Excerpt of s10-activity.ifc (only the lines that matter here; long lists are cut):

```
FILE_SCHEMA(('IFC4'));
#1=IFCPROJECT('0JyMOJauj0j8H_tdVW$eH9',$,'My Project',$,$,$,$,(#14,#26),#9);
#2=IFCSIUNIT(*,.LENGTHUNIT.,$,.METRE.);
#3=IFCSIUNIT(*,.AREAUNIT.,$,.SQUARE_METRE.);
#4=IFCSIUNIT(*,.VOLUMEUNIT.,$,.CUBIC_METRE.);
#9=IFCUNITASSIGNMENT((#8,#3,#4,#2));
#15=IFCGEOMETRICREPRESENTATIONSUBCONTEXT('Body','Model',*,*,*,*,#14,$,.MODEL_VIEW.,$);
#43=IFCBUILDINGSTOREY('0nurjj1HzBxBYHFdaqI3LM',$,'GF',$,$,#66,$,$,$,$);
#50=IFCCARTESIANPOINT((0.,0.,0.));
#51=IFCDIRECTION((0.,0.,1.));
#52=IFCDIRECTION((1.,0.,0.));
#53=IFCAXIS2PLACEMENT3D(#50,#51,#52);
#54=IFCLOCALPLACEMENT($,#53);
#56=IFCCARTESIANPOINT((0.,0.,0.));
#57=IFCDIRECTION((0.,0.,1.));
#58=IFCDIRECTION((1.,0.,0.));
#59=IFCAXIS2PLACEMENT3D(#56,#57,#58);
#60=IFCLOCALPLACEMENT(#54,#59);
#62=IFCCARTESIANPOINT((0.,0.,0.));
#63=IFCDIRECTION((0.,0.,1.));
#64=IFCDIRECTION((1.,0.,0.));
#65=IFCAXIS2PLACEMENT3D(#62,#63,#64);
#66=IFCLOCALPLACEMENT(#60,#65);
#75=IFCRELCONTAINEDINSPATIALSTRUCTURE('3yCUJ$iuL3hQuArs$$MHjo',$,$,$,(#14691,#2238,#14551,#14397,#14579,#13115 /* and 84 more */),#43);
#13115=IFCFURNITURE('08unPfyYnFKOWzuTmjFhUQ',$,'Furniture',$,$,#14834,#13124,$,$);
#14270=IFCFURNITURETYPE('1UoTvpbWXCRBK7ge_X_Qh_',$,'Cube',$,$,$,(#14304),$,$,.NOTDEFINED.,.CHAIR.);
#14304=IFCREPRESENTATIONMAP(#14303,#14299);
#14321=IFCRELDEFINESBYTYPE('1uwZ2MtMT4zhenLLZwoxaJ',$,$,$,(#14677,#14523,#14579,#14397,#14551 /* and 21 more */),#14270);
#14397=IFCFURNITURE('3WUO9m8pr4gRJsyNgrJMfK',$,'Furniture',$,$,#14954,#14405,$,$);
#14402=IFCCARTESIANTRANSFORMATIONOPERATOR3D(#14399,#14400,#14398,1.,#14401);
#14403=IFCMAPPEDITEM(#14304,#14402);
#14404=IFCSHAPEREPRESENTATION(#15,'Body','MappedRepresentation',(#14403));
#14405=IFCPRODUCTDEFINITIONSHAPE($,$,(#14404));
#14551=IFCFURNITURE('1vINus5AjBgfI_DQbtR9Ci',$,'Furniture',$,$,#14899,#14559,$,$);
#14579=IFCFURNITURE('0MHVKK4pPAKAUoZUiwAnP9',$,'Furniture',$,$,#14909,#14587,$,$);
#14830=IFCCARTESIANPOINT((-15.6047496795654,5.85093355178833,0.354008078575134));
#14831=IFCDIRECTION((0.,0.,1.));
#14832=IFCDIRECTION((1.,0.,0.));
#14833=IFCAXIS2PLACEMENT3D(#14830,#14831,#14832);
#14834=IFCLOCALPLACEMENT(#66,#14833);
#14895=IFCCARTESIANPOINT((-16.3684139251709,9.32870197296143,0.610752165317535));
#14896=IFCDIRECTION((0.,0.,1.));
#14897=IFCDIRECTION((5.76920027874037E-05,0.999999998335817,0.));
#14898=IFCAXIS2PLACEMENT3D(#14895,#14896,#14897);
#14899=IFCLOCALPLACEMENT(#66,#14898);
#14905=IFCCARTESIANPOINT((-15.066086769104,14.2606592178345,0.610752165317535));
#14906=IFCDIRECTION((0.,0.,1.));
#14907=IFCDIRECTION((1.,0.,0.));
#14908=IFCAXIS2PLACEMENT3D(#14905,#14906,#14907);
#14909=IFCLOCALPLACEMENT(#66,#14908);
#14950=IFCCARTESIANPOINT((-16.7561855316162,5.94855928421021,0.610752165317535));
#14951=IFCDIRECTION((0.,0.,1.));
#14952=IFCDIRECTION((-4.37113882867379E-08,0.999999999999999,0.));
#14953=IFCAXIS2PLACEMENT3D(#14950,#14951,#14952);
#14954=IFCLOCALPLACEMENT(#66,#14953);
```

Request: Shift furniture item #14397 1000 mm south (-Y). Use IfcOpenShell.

```python
import ifcopenshell
import ifcopenshell.api.geometry
import ifcopenshell.util.placement

model = ifcopenshell.open("s10-activity.ifc")

item = model.by_id(14397)
matrix = ifcopenshell.util.placement.get_local_placement(item.ObjectPlacement)
matrix[1, 3] -= 1.0
ifcopenshell.api.geometry.edit_object_placement(model, product=item, matrix=matrix, is_si=False)

print(ifcopenshell.util.placement.get_local_placement(item.ObjectPlacement).round(3) + 0.0)

model.write("s10-activity_v2.ifc")
```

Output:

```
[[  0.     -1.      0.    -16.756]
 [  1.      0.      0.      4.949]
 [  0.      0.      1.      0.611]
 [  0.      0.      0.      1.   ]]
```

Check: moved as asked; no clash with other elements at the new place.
